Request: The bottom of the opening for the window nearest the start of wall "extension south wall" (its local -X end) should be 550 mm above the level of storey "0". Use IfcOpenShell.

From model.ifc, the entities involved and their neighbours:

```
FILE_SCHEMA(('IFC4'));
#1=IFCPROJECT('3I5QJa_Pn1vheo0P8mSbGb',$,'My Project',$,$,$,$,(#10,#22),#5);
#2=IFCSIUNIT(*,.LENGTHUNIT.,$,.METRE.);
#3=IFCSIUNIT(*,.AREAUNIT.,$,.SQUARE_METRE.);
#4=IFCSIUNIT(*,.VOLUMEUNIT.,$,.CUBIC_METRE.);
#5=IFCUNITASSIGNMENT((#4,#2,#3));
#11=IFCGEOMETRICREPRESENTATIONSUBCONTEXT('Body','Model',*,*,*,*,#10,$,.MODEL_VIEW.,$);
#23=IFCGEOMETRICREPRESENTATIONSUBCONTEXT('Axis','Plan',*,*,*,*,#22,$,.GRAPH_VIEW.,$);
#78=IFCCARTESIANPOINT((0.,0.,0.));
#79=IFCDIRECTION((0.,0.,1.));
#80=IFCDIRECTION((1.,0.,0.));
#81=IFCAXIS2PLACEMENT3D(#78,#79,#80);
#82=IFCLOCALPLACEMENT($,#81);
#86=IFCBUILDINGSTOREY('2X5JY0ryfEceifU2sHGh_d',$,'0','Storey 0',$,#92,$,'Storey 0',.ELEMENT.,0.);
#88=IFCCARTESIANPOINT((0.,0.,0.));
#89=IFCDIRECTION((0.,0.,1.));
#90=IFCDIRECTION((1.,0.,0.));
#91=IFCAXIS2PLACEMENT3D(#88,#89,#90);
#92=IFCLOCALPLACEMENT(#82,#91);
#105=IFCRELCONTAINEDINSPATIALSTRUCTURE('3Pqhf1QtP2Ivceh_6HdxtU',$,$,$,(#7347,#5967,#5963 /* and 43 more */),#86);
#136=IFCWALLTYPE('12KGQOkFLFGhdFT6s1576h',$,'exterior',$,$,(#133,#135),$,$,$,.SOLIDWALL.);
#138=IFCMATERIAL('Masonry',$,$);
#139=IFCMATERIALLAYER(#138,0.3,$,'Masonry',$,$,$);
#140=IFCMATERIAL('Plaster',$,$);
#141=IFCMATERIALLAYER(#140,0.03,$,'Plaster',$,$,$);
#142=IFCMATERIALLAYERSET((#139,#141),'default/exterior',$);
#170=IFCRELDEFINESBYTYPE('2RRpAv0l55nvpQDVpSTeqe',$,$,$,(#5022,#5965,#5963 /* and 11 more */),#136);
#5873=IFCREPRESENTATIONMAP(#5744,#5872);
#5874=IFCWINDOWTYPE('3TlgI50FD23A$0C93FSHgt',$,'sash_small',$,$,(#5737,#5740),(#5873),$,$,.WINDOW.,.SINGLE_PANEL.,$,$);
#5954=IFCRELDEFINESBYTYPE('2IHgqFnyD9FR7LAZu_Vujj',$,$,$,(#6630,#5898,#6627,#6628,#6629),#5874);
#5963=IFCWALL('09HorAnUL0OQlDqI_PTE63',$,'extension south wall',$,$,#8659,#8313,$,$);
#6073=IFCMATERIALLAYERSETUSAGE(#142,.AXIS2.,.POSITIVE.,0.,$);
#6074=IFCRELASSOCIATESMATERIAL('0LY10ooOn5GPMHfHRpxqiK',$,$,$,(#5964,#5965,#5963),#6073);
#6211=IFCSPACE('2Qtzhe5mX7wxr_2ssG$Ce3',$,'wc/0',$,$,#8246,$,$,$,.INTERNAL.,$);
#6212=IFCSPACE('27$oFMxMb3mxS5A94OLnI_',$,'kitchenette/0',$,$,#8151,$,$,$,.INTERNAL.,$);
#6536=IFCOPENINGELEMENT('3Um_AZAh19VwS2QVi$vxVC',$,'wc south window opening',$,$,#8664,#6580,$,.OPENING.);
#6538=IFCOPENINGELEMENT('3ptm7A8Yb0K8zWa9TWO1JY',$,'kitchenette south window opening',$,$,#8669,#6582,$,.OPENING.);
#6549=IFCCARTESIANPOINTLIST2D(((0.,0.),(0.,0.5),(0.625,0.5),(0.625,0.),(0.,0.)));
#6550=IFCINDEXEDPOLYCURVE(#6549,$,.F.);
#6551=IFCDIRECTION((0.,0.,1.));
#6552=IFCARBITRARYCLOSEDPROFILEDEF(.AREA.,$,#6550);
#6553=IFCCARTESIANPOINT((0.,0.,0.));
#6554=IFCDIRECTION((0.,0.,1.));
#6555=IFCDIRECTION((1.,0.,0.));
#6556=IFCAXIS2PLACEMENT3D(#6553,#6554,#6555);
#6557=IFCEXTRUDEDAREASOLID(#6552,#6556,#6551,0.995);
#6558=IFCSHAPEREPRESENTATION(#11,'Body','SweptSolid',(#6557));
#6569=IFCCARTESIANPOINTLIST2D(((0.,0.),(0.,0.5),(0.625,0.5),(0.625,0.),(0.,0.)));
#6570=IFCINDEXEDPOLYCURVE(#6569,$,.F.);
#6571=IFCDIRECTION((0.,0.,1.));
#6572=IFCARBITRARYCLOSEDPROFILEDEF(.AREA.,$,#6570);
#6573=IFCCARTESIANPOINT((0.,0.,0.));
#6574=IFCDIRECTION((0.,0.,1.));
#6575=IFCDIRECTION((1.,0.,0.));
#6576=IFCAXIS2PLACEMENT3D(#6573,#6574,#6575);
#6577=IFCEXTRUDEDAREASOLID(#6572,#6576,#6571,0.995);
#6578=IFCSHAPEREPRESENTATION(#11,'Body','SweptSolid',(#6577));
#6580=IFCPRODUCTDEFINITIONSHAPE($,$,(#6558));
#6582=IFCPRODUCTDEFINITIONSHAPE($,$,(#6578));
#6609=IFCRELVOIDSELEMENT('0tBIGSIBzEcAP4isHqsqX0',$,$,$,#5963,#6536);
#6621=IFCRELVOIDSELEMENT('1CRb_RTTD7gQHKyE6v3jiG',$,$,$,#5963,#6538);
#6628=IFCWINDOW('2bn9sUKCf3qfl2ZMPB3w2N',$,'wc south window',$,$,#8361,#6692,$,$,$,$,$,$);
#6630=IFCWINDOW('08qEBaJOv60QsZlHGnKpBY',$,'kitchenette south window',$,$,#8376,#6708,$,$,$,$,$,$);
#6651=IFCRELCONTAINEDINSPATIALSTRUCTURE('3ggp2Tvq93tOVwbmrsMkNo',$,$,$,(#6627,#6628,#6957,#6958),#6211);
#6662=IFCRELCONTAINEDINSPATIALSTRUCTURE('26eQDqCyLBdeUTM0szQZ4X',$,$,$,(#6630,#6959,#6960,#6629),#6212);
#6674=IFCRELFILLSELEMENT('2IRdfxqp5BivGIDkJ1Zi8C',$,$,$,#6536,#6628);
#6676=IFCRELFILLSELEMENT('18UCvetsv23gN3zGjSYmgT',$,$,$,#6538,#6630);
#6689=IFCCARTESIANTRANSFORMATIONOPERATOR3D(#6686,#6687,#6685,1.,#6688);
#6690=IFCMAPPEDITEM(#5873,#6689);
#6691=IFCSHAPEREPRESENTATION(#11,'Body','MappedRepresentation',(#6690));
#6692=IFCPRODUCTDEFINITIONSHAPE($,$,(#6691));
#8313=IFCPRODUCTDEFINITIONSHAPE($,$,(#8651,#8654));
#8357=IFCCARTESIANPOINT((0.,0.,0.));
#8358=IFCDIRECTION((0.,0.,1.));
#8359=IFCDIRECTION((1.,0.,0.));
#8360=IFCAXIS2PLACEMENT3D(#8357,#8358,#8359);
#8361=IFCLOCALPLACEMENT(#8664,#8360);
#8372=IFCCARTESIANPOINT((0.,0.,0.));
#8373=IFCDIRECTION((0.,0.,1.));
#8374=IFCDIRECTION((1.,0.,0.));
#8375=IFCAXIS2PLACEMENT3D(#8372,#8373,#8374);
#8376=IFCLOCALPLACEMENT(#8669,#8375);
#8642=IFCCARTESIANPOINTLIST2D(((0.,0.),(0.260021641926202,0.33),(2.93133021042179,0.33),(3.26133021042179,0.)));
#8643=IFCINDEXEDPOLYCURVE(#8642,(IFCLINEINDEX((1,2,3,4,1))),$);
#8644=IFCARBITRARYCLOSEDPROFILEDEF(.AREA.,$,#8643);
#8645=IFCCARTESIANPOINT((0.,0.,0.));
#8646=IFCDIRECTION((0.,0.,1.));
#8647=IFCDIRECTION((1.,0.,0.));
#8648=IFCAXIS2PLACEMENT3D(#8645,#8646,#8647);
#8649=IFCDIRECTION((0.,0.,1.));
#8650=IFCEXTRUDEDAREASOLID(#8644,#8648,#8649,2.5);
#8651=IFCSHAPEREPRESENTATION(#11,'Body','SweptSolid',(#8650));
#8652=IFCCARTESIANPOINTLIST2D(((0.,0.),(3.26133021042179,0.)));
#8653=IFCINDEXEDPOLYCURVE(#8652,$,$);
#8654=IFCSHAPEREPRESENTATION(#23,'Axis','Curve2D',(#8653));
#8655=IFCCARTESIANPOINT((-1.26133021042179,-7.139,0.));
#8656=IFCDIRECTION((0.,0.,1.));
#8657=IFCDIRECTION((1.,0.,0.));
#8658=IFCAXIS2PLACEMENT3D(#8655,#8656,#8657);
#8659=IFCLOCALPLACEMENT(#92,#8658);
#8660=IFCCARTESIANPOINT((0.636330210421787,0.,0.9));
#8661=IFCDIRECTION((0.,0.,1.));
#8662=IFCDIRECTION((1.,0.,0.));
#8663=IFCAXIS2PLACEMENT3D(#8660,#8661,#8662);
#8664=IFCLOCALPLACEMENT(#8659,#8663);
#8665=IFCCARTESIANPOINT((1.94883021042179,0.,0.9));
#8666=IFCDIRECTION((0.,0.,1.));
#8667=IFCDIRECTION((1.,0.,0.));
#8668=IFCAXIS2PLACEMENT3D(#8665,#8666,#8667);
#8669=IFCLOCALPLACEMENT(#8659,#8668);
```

```python
import numpy as np
import ifcopenshell
import ifcopenshell.api.geometry
import ifcopenshell.geom
import ifcopenshell.util.element
import ifcopenshell.util.placement
import ifcopenshell.util.shape
import ifcopenshell.util.unit

model = ifcopenshell.open("model.ifc")
unit_scale = ifcopenshell.util.unit.calculate_unit_scale(model)

window = model.by_guid("2bn9sUKCf3qfl2ZMPB3w2N")
opening = window.FillsVoids[0].RelatingOpeningElement
storey = ifcopenshell.util.element.get_container(window, ifc_class="IfcBuildingStorey")
level = ifcopenshell.util.placement.get_local_placement(storey.ObjectPlacement)[2, 3]

# The opening's origin need not be at the sill, so measure its lowest point.
shape = ifcopenshell.geom.create_shape(ifcopenshell.geom.settings(), opening)
bottom = ifcopenshell.util.shape.get_shape_bottom_elevation(shape, shape.geometry) / unit_scale
dz = level + 0.55 - bottom

shift = np.array([0.0, 0.0, dz])
# The window is placed relative to its opening, so it follows when the opening moves.
matrix = ifcopenshell.util.placement.get_local_placement(opening.ObjectPlacement)
matrix[:3, 3] += shift
ifcopenshell.api.geometry.edit_object_placement(
    model, product=opening, matrix=matrix, is_si=False, should_transform_children=True
)

print(f"moved by {dz * unit_scale:+.3f} m")

model.write("model_rev.ifc")
```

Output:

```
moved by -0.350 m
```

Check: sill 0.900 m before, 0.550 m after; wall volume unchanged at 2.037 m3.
